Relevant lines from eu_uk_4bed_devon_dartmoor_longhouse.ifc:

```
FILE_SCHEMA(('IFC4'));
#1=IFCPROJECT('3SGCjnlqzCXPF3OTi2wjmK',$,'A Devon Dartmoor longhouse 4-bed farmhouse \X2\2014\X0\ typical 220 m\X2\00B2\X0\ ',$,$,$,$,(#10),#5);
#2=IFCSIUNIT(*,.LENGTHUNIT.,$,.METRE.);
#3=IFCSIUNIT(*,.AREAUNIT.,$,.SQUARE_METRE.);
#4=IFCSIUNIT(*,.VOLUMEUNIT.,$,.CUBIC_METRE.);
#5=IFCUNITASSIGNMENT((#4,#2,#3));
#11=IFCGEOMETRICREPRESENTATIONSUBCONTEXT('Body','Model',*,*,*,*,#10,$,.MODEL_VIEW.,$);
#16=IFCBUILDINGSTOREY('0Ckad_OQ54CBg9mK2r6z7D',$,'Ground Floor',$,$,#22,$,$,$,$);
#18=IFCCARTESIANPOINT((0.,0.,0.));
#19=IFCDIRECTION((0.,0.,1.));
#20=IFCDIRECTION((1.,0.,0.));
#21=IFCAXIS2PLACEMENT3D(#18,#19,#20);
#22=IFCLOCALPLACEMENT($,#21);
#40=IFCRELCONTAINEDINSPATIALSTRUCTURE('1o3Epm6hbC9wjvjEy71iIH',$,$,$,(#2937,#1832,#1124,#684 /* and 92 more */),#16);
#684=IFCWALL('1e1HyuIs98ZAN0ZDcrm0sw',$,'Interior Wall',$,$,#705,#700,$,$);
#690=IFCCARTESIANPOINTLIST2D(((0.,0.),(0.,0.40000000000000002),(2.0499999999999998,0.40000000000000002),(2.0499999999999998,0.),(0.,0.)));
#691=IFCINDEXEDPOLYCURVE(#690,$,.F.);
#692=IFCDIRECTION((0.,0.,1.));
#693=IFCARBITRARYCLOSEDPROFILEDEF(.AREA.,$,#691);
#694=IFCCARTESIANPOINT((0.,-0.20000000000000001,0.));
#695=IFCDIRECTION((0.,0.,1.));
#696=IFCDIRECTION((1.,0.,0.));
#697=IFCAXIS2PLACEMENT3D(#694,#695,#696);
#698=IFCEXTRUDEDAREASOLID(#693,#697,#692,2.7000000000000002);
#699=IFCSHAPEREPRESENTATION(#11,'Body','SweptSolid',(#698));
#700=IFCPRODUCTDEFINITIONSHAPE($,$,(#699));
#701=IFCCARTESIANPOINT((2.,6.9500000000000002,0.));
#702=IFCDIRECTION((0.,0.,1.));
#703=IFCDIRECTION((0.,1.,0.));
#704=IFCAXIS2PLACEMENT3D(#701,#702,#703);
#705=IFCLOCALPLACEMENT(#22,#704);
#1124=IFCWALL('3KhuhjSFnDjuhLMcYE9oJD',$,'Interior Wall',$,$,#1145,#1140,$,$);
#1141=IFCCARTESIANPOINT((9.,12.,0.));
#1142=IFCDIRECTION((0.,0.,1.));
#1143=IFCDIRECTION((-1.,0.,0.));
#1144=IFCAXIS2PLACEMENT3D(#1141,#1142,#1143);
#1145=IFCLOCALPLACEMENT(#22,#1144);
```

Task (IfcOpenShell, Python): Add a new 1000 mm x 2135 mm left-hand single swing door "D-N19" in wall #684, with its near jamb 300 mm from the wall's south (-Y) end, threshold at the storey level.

```python
import numpy as np
import ifcopenshell
import ifcopenshell.api.feature
import ifcopenshell.api.geometry
import ifcopenshell.api.root
import ifcopenshell.api.spatial
import ifcopenshell.geom
import ifcopenshell.util.element
import ifcopenshell.util.placement
import ifcopenshell.util.representation
import ifcopenshell.util.shape
import ifcopenshell.util.unit

model = ifcopenshell.open("eu_uk_4bed_devon_dartmoor_longhouse.ifc")
unit_scale = ifcopenshell.util.unit.calculate_unit_scale(model)
settings = ifcopenshell.geom.settings()


def volume(element):
    """Net volume in cubic metres, openings subtracted."""
    shape = ifcopenshell.geom.create_shape(settings, element)
    return ifcopenshell.util.shape.get_volume(shape.geometry)


wall = model.by_guid("1e1HyuIs98ZAN0ZDcrm0sw")
storey = ifcopenshell.util.element.get_container(wall, ifc_class="IfcBuildingStorey")
context = ifcopenshell.util.representation.get_context(model, "Model", "Body", "MODEL_VIEW")
before = volume(wall)

width, height, from_end, sill = 1, 2.135, 0.3, 0.0  # metres

# The wall runs along its own X axis, and the end named is its -X end.
wall_shape = ifcopenshell.geom.create_shape(settings, wall)
x, y, z = ifcopenshell.util.shape.get_vertices(wall_shape.geometry).T
start = x.min() + from_end
face, thickness = float(y.min()), float(y.max() - y.min())
wall_matrix = ifcopenshell.util.placement.get_local_placement(wall.ObjectPlacement)
level = ifcopenshell.util.placement.get_local_placement(storey.ObjectPlacement)[2, 3]


def in_wall(x, y):
    """Placement at x, y metres in the wall's axes, at sill height."""
    matrix = wall_matrix.copy()
    matrix[:, 3] = wall_matrix @ np.array([x / unit_scale, y / unit_scale, 0.0, 1.0])
    matrix[2, 3] = level + sill / unit_scale
    return matrix


# Opening: a box that overshoots both wall faces by 50 mm.
opening = ifcopenshell.api.root.create_entity(model, ifc_class="IfcOpeningElement", predefined_type="OPENING")
box = ifcopenshell.api.geometry.add_wall_representation(
    model, context=context, length=width, height=height, thickness=thickness + 0.1
)
ifcopenshell.api.geometry.assign_representation(model, product=opening, representation=box)
ifcopenshell.api.geometry.edit_object_placement(model, product=opening, matrix=in_wall(start, face - 0.05), is_si=False)
ifcopenshell.api.feature.add_feature(model, feature=opening, element=wall)

door = ifcopenshell.api.root.create_entity(model, ifc_class="IfcDoor", name="D-N19", predefined_type="DOOR")
door.OverallWidth, door.OverallHeight = width / unit_scale, height / unit_scale
door.OperationType = "SINGLE_SWING_LEFT"
body = ifcopenshell.api.geometry.add_door_representation(
    model,
    context=context,
    overall_width=door.OverallWidth,
    overall_height=door.OverallHeight,
    operation_type="SINGLE_SWING_LEFT",
    lining_properties={"LiningDepth": thickness / unit_scale, "ThresholdDepth": thickness / unit_scale},
)
ifcopenshell.api.geometry.assign_representation(model, product=door, representation=body)
ifcopenshell.api.spatial.assign_container(model, products=[door], relating_structure=storey)
ifcopenshell.api.feature.add_filling(model, opening=opening, element=door)

# The lining spans the wall, so the door starts at the wall face.
ifcopenshell.api.geometry.edit_object_placement(model, product=door, matrix=in_wall(start, face), is_si=False)

after = volume(wall)

print(f"wall volume {before:.3f} -> {after:.3f} m3")

model.write("eu_uk_4bed_devon_dartmoor_longhouse_edited.ifc")
```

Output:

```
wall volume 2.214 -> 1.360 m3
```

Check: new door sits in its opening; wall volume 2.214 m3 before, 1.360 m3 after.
